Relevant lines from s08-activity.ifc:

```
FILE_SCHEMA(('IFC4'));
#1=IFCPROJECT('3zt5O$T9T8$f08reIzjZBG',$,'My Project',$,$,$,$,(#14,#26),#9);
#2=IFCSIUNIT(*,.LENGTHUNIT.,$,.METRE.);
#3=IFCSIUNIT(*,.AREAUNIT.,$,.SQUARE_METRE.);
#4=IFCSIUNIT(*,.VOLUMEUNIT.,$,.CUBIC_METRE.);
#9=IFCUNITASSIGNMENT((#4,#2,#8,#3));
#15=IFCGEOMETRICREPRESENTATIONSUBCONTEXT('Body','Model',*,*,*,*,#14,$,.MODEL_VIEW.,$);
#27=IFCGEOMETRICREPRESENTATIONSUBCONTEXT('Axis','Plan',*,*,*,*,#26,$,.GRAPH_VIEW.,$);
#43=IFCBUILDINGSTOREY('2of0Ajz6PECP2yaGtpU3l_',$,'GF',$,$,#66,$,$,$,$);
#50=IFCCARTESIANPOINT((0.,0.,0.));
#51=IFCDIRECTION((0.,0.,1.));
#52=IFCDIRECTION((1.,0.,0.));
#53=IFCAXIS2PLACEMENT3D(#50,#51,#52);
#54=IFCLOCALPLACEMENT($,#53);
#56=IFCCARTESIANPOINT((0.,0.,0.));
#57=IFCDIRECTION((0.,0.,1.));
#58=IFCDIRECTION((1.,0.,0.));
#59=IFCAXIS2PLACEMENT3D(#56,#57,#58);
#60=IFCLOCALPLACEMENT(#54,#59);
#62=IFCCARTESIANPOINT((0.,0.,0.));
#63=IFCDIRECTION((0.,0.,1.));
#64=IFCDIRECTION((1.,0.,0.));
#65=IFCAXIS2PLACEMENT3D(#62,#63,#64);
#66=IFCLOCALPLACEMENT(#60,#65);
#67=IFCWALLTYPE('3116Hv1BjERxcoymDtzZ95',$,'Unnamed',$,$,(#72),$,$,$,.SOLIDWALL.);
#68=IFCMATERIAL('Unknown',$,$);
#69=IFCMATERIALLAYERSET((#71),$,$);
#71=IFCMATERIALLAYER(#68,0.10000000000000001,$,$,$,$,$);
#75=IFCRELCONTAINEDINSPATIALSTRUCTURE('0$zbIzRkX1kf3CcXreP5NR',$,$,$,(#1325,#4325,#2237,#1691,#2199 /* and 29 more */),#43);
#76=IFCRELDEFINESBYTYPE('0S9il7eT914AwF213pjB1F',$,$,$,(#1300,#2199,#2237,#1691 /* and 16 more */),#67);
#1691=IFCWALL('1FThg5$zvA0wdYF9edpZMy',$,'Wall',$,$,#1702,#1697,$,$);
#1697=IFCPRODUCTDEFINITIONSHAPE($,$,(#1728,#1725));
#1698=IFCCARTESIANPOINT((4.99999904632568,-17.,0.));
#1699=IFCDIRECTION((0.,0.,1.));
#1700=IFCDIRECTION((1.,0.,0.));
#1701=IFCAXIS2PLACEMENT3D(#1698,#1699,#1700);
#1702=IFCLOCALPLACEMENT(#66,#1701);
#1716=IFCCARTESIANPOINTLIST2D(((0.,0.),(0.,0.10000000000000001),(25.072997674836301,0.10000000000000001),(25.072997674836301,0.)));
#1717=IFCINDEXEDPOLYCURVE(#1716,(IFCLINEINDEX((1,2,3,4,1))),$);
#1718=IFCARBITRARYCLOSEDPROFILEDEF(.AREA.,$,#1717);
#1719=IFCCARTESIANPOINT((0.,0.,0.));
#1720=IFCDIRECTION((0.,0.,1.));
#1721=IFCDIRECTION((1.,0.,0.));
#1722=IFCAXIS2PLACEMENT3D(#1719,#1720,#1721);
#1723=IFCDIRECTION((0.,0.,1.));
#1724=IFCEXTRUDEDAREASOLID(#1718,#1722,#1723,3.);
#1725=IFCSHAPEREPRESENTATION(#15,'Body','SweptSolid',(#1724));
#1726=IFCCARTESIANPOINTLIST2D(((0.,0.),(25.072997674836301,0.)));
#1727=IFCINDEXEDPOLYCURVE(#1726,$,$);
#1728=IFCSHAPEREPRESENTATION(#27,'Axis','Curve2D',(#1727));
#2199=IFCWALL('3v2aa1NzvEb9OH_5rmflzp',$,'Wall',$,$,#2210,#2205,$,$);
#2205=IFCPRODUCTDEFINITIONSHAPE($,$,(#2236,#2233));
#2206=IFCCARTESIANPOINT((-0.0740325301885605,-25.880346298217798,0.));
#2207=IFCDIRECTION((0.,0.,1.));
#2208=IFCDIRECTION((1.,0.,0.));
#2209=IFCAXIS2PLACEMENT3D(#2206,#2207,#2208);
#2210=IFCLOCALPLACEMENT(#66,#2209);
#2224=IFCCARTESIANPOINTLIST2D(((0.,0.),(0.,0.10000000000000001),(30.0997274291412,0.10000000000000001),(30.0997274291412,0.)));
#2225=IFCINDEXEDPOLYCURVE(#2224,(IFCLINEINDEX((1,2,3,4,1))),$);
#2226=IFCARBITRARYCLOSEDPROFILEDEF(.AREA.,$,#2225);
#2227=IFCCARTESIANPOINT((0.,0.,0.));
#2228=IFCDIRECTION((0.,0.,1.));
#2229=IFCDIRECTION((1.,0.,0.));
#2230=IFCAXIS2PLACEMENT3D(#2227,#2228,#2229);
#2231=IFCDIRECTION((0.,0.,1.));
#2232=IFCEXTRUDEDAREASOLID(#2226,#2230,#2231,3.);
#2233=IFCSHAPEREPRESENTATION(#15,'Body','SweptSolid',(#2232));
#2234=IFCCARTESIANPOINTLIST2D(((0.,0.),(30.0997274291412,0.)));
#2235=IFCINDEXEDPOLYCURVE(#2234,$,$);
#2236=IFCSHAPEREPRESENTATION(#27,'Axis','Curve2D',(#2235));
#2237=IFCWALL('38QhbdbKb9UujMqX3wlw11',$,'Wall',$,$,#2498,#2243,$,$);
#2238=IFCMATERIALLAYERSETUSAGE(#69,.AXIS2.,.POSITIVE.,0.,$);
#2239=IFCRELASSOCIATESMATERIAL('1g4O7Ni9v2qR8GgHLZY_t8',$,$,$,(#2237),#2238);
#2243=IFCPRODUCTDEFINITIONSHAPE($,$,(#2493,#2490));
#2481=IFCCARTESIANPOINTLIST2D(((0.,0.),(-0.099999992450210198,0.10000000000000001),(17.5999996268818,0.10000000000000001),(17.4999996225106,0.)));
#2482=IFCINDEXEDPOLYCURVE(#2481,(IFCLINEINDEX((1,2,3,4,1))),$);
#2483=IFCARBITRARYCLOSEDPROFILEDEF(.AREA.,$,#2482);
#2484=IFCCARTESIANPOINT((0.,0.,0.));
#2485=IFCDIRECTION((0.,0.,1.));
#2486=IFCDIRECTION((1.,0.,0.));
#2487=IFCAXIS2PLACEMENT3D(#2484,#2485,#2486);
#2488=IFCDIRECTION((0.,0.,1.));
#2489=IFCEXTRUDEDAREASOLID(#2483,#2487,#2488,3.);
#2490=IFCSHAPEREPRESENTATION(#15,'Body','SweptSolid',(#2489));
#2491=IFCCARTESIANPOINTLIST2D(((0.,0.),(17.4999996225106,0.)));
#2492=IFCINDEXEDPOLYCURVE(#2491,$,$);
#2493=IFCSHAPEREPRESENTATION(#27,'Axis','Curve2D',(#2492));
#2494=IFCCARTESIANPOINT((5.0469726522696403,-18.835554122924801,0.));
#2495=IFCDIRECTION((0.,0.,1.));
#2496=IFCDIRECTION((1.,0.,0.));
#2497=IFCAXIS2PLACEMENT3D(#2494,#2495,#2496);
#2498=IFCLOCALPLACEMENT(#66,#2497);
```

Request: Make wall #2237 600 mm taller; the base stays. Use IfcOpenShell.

```python
import ifcopenshell
import ifcopenshell.geom
import ifcopenshell.util.representation
import ifcopenshell.util.shape
import ifcopenshell.util.unit

model = ifcopenshell.open("s08-activity.ifc")
unit_scale = ifcopenshell.util.unit.calculate_unit_scale(model)
settings = ifcopenshell.geom.settings()


def volume(element):
    """Net volume in cubic metres, openings subtracted."""
    shape = ifcopenshell.geom.create_shape(settings, element)
    return ifcopenshell.util.shape.get_volume(shape.geometry)


wall = model.by_id(2237)
before = volume(wall)

body = ifcopenshell.util.representation.get_representation(wall, "Model", "Body")
solid = body.Items[0]
old_height = solid.Depth
solid.Depth += 0.6 / unit_scale
after = volume(wall)

print(f"height {old_height:g} -> {solid.Depth:g}, volume {before:.3f} -> {after:.3f} m3")

model.write("s08-activity_rev.ifc")
```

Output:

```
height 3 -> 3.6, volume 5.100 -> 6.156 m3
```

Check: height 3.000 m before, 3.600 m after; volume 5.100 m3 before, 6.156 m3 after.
